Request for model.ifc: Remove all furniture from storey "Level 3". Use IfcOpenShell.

First a look at what the model holds.

```python
import ifcopenshell
import ifcopenshell.util.element

model = ifcopenshell.open("model.ifc")
print(model.schema)
storey = next(s for s in model.by_type("IfcBuildingStorey") if s.Name == "Level 3")
furniture = [e for e in ifcopenshell.util.element.get_decomposition(storey) if e.is_a("IfcFurnishingElement")]
seen = {}
for e in furniture:
    element_type = ifcopenshell.util.element.get_type(e)
    name = element_type.Name if element_type not in (None, e) else None
    seen[name] = seen.get(name, 0) + 1
for name, count in sorted(seen.items(), key=str):
    print(count, "x", name)
```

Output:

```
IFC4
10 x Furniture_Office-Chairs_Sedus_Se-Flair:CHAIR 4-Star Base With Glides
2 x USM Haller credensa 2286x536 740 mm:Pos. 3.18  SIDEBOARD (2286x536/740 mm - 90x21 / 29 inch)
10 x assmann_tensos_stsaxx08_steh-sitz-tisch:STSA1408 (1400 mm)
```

```python
import ifcopenshell
import ifcopenshell.api.root
import ifcopenshell.util.element

model = ifcopenshell.open("model.ifc")

storey = next(s for s in model.by_type("IfcBuildingStorey") if s.Name == "Level 3")
furniture = [e for e in ifcopenshell.util.element.get_decomposition(storey) if e.is_a("IfcFurnishingElement")]

for e in furniture:
    ifcopenshell.api.root.remove_product(model, product=e)
print(len(furniture), "removed")

model.write("model-out.ifc")
```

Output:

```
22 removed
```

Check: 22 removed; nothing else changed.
